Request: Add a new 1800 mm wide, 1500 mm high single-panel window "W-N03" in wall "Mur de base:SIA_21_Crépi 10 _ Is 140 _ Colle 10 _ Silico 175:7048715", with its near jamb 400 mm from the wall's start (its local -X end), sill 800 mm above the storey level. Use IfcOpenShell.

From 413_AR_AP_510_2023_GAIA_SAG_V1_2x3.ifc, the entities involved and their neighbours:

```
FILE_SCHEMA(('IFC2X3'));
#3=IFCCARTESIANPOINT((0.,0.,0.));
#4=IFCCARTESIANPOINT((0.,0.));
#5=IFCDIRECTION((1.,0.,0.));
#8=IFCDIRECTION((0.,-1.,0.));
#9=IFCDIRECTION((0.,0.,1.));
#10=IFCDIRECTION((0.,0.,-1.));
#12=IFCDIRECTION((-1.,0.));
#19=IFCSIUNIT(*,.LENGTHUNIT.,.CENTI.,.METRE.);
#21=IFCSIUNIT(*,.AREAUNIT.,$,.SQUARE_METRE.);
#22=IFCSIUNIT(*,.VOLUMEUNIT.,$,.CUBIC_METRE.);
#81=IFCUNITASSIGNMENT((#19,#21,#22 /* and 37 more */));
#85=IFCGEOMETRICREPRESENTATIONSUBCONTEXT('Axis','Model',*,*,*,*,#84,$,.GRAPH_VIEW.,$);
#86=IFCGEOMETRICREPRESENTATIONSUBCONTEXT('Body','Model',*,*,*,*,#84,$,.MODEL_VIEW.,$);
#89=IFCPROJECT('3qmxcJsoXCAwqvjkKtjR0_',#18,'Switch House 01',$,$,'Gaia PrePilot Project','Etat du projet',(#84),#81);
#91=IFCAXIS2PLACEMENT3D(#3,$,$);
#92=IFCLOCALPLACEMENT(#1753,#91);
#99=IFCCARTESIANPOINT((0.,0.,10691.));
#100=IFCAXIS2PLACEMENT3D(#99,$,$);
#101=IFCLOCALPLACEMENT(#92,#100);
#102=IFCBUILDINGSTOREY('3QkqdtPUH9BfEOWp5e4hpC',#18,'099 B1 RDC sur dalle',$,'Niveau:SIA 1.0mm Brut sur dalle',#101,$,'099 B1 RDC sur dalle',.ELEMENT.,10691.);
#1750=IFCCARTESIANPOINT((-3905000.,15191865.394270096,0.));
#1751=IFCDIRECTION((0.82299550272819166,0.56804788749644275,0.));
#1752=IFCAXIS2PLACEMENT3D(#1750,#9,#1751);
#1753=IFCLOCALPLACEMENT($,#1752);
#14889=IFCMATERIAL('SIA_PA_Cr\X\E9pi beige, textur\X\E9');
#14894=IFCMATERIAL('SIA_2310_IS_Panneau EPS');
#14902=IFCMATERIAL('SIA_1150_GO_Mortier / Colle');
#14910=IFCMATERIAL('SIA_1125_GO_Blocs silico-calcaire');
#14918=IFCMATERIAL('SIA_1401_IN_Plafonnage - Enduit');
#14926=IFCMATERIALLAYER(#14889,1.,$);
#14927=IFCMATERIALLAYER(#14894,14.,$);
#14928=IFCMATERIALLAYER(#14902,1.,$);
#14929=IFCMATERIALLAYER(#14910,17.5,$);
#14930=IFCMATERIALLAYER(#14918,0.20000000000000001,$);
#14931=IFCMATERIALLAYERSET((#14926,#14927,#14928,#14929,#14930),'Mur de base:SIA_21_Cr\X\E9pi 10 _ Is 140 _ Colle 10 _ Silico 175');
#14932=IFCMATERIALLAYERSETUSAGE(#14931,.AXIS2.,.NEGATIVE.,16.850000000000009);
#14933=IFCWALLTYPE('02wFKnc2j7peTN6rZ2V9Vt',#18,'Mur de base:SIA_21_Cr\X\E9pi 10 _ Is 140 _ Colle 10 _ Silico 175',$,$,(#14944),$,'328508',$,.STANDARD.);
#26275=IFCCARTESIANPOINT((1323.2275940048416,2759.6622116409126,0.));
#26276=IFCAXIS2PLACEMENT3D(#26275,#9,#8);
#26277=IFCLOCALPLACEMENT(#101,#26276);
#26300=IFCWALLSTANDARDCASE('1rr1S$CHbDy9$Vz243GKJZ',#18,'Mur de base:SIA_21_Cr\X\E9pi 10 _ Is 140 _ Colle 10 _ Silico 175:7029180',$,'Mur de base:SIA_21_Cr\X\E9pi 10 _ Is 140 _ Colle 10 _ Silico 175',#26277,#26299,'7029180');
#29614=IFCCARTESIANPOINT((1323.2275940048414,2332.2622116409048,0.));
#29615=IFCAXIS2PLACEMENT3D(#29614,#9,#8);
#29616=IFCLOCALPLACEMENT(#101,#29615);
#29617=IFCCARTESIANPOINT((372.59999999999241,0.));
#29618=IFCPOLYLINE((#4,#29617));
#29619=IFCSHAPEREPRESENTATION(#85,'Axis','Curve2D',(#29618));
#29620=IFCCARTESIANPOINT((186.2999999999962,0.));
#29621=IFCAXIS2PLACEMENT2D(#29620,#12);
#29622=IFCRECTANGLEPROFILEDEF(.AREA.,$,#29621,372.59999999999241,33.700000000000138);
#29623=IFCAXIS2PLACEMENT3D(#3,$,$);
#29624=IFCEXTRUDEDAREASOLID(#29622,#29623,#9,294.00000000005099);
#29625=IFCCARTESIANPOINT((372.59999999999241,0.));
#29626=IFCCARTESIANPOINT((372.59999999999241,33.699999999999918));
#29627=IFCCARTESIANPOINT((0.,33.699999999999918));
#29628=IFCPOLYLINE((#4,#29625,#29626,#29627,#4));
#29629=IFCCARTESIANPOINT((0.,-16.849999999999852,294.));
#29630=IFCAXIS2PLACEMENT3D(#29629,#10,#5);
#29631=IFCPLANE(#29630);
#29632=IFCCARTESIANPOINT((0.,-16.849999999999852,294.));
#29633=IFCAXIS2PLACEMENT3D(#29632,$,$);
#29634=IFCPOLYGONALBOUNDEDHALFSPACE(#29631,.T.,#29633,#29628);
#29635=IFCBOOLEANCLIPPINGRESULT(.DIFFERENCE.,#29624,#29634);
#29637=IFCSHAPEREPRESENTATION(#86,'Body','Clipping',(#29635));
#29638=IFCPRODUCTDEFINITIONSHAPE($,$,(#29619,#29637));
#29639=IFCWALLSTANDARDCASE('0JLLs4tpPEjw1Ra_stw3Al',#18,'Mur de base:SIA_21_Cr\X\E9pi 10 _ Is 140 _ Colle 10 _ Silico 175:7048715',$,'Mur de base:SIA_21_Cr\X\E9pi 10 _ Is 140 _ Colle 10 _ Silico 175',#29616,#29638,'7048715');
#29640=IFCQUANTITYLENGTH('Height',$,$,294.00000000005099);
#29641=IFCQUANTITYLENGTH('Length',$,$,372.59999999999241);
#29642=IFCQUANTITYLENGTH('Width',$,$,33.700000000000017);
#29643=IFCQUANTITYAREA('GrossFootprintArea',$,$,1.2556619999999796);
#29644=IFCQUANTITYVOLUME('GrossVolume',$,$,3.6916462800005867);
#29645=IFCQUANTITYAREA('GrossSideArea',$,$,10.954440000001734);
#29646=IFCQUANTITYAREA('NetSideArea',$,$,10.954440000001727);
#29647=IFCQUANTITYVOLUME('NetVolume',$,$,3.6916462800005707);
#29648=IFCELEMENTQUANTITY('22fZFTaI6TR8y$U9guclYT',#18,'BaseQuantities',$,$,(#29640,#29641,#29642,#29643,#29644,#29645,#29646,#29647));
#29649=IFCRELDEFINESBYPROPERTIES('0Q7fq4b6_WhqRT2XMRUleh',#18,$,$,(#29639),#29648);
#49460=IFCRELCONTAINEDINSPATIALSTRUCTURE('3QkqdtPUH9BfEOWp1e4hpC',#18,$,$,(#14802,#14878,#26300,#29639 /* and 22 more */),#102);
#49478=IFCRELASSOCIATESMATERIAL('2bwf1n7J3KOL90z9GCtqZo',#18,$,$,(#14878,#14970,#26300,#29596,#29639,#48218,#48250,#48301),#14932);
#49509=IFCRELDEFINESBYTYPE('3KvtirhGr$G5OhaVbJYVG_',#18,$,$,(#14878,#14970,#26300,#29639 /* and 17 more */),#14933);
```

```python
import numpy as np
import ifcopenshell
import ifcopenshell.api.feature
import ifcopenshell.api.geometry
import ifcopenshell.api.pset
import ifcopenshell.api.root
import ifcopenshell.api.spatial
import ifcopenshell.api.type
import ifcopenshell.geom
import ifcopenshell.util.element
import ifcopenshell.util.placement
import ifcopenshell.util.representation
import ifcopenshell.util.shape
import ifcopenshell.util.unit

model = ifcopenshell.open("413_AR_AP_510_2023_GAIA_SAG_V1_2x3.ifc")
unit_scale = ifcopenshell.util.unit.calculate_unit_scale(model)
area_scale = ifcopenshell.util.unit.calculate_unit_scale(model, "AREAUNIT")
volume_scale = ifcopenshell.util.unit.calculate_unit_scale(model, "VOLUMEUNIT")
settings = ifcopenshell.geom.settings()


def volume(element):
    """Net volume in cubic metres, openings subtracted."""
    shape = ifcopenshell.geom.create_shape(settings, element)
    return ifcopenshell.util.shape.get_volume(shape.geometry)


wall = model.by_guid("0JLLs4tpPEjw1Ra_stw3Al")
storey = ifcopenshell.util.element.get_container(wall, ifc_class="IfcBuildingStorey")
context = ifcopenshell.util.representation.get_context(model, "Model", "Body", "MODEL_VIEW")
before = volume(wall)

width, height, from_end, sill = 1.8, 1.5, 0.4, 0.8  # metres

# The wall runs along its own X axis, and the end named is its -X end.
wall_shape = ifcopenshell.geom.create_shape(settings, wall)
x, y, z = ifcopenshell.util.shape.get_vertices(wall_shape.geometry).T
start = x.min() + from_end
face, thickness = float(y.min()), float(y.max() - y.min())
wall_matrix = ifcopenshell.util.placement.get_local_placement(wall.ObjectPlacement)
level = ifcopenshell.util.placement.get_local_placement(storey.ObjectPlacement)[2, 3]


def in_wall(x, y):
    """Placement at x, y metres in the wall's axes, at sill height."""
    matrix = wall_matrix.copy()
    matrix[:, 3] = wall_matrix @ np.array([x / unit_scale, y / unit_scale, 0.0, 1.0])
    matrix[2, 3] = level + sill / unit_scale
    return matrix


# Opening: a box that overshoots both wall faces by 50 mm.
opening = ifcopenshell.api.root.create_entity(model, ifc_class="IfcOpeningElement")
box = ifcopenshell.api.geometry.add_wall_representation(
    model, context=context, length=width, height=height, thickness=thickness + 0.1
)
ifcopenshell.api.geometry.assign_representation(model, product=opening, representation=box)
ifcopenshell.api.geometry.edit_object_placement(model, product=opening, matrix=in_wall(start, face - 0.05), is_si=False)
ifcopenshell.api.feature.add_feature(model, feature=opening, element=wall)

window = ifcopenshell.api.root.create_entity(model, ifc_class="IfcWindow", name="W-N03")
window.OverallWidth, window.OverallHeight = width / unit_scale, height / unit_scale
body = ifcopenshell.api.geometry.add_window_representation(
    model,
    context=context,
    overall_width=window.OverallWidth,
    overall_height=window.OverallHeight,
    partition_type="SINGLE_PANEL",
)
ifcopenshell.api.geometry.assign_representation(model, product=window, representation=body)
ifcopenshell.api.spatial.assign_container(model, products=[window], relating_structure=storey)
fills = ifcopenshell.api.feature.add_filling(model, opening=opening, element=window)
fills.OwnerHistory = window.OwnerHistory  # required in IFC2X3

# IFC2X3 keeps the operation on the window style.
style = ifcopenshell.api.root.create_entity(model, ifc_class="IfcWindowStyle", name="W-N03")
style.OperationType, style.ConstructionType = "SINGLE_PANEL", "NOTDEFINED"
style.ParameterTakesPrecedence = style.Sizeable = False
ifcopenshell.api.type.assign_type(model, related_objects=[window], relating_type=style)

# Centre the window in the wall's thickness.
ifcopenshell.api.geometry.edit_object_placement(model, product=window, matrix=in_wall(start, face), is_si=False)
window_shape = ifcopenshell.geom.create_shape(settings, window)
depth = ifcopenshell.util.shape.get_vertices(window_shape.geometry)[:, 1]
offset = face + thickness / 2 - (depth.min() + depth.max()) / 2
ifcopenshell.api.geometry.edit_object_placement(model, product=window, matrix=in_wall(start, offset), is_si=False)

after = volume(wall)

# Update the wall's stored quantities.
qto = model.by_id(ifcopenshell.util.element.get_pset(wall, "BaseQuantities", should_inherit=False)["id"])
ifcopenshell.api.pset.edit_qto(model, qto=qto, properties={
    "NetSideArea": after / thickness / area_scale,
    "NetVolume": after / volume_scale,
})

print(f"wall volume {before:.3f} -> {after:.3f} m3")

model.write("413_AR_AP_510_2023_GAIA_SAG_V1_2x3_rev.ifc")
```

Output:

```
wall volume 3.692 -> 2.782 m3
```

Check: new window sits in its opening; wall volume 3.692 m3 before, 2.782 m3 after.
